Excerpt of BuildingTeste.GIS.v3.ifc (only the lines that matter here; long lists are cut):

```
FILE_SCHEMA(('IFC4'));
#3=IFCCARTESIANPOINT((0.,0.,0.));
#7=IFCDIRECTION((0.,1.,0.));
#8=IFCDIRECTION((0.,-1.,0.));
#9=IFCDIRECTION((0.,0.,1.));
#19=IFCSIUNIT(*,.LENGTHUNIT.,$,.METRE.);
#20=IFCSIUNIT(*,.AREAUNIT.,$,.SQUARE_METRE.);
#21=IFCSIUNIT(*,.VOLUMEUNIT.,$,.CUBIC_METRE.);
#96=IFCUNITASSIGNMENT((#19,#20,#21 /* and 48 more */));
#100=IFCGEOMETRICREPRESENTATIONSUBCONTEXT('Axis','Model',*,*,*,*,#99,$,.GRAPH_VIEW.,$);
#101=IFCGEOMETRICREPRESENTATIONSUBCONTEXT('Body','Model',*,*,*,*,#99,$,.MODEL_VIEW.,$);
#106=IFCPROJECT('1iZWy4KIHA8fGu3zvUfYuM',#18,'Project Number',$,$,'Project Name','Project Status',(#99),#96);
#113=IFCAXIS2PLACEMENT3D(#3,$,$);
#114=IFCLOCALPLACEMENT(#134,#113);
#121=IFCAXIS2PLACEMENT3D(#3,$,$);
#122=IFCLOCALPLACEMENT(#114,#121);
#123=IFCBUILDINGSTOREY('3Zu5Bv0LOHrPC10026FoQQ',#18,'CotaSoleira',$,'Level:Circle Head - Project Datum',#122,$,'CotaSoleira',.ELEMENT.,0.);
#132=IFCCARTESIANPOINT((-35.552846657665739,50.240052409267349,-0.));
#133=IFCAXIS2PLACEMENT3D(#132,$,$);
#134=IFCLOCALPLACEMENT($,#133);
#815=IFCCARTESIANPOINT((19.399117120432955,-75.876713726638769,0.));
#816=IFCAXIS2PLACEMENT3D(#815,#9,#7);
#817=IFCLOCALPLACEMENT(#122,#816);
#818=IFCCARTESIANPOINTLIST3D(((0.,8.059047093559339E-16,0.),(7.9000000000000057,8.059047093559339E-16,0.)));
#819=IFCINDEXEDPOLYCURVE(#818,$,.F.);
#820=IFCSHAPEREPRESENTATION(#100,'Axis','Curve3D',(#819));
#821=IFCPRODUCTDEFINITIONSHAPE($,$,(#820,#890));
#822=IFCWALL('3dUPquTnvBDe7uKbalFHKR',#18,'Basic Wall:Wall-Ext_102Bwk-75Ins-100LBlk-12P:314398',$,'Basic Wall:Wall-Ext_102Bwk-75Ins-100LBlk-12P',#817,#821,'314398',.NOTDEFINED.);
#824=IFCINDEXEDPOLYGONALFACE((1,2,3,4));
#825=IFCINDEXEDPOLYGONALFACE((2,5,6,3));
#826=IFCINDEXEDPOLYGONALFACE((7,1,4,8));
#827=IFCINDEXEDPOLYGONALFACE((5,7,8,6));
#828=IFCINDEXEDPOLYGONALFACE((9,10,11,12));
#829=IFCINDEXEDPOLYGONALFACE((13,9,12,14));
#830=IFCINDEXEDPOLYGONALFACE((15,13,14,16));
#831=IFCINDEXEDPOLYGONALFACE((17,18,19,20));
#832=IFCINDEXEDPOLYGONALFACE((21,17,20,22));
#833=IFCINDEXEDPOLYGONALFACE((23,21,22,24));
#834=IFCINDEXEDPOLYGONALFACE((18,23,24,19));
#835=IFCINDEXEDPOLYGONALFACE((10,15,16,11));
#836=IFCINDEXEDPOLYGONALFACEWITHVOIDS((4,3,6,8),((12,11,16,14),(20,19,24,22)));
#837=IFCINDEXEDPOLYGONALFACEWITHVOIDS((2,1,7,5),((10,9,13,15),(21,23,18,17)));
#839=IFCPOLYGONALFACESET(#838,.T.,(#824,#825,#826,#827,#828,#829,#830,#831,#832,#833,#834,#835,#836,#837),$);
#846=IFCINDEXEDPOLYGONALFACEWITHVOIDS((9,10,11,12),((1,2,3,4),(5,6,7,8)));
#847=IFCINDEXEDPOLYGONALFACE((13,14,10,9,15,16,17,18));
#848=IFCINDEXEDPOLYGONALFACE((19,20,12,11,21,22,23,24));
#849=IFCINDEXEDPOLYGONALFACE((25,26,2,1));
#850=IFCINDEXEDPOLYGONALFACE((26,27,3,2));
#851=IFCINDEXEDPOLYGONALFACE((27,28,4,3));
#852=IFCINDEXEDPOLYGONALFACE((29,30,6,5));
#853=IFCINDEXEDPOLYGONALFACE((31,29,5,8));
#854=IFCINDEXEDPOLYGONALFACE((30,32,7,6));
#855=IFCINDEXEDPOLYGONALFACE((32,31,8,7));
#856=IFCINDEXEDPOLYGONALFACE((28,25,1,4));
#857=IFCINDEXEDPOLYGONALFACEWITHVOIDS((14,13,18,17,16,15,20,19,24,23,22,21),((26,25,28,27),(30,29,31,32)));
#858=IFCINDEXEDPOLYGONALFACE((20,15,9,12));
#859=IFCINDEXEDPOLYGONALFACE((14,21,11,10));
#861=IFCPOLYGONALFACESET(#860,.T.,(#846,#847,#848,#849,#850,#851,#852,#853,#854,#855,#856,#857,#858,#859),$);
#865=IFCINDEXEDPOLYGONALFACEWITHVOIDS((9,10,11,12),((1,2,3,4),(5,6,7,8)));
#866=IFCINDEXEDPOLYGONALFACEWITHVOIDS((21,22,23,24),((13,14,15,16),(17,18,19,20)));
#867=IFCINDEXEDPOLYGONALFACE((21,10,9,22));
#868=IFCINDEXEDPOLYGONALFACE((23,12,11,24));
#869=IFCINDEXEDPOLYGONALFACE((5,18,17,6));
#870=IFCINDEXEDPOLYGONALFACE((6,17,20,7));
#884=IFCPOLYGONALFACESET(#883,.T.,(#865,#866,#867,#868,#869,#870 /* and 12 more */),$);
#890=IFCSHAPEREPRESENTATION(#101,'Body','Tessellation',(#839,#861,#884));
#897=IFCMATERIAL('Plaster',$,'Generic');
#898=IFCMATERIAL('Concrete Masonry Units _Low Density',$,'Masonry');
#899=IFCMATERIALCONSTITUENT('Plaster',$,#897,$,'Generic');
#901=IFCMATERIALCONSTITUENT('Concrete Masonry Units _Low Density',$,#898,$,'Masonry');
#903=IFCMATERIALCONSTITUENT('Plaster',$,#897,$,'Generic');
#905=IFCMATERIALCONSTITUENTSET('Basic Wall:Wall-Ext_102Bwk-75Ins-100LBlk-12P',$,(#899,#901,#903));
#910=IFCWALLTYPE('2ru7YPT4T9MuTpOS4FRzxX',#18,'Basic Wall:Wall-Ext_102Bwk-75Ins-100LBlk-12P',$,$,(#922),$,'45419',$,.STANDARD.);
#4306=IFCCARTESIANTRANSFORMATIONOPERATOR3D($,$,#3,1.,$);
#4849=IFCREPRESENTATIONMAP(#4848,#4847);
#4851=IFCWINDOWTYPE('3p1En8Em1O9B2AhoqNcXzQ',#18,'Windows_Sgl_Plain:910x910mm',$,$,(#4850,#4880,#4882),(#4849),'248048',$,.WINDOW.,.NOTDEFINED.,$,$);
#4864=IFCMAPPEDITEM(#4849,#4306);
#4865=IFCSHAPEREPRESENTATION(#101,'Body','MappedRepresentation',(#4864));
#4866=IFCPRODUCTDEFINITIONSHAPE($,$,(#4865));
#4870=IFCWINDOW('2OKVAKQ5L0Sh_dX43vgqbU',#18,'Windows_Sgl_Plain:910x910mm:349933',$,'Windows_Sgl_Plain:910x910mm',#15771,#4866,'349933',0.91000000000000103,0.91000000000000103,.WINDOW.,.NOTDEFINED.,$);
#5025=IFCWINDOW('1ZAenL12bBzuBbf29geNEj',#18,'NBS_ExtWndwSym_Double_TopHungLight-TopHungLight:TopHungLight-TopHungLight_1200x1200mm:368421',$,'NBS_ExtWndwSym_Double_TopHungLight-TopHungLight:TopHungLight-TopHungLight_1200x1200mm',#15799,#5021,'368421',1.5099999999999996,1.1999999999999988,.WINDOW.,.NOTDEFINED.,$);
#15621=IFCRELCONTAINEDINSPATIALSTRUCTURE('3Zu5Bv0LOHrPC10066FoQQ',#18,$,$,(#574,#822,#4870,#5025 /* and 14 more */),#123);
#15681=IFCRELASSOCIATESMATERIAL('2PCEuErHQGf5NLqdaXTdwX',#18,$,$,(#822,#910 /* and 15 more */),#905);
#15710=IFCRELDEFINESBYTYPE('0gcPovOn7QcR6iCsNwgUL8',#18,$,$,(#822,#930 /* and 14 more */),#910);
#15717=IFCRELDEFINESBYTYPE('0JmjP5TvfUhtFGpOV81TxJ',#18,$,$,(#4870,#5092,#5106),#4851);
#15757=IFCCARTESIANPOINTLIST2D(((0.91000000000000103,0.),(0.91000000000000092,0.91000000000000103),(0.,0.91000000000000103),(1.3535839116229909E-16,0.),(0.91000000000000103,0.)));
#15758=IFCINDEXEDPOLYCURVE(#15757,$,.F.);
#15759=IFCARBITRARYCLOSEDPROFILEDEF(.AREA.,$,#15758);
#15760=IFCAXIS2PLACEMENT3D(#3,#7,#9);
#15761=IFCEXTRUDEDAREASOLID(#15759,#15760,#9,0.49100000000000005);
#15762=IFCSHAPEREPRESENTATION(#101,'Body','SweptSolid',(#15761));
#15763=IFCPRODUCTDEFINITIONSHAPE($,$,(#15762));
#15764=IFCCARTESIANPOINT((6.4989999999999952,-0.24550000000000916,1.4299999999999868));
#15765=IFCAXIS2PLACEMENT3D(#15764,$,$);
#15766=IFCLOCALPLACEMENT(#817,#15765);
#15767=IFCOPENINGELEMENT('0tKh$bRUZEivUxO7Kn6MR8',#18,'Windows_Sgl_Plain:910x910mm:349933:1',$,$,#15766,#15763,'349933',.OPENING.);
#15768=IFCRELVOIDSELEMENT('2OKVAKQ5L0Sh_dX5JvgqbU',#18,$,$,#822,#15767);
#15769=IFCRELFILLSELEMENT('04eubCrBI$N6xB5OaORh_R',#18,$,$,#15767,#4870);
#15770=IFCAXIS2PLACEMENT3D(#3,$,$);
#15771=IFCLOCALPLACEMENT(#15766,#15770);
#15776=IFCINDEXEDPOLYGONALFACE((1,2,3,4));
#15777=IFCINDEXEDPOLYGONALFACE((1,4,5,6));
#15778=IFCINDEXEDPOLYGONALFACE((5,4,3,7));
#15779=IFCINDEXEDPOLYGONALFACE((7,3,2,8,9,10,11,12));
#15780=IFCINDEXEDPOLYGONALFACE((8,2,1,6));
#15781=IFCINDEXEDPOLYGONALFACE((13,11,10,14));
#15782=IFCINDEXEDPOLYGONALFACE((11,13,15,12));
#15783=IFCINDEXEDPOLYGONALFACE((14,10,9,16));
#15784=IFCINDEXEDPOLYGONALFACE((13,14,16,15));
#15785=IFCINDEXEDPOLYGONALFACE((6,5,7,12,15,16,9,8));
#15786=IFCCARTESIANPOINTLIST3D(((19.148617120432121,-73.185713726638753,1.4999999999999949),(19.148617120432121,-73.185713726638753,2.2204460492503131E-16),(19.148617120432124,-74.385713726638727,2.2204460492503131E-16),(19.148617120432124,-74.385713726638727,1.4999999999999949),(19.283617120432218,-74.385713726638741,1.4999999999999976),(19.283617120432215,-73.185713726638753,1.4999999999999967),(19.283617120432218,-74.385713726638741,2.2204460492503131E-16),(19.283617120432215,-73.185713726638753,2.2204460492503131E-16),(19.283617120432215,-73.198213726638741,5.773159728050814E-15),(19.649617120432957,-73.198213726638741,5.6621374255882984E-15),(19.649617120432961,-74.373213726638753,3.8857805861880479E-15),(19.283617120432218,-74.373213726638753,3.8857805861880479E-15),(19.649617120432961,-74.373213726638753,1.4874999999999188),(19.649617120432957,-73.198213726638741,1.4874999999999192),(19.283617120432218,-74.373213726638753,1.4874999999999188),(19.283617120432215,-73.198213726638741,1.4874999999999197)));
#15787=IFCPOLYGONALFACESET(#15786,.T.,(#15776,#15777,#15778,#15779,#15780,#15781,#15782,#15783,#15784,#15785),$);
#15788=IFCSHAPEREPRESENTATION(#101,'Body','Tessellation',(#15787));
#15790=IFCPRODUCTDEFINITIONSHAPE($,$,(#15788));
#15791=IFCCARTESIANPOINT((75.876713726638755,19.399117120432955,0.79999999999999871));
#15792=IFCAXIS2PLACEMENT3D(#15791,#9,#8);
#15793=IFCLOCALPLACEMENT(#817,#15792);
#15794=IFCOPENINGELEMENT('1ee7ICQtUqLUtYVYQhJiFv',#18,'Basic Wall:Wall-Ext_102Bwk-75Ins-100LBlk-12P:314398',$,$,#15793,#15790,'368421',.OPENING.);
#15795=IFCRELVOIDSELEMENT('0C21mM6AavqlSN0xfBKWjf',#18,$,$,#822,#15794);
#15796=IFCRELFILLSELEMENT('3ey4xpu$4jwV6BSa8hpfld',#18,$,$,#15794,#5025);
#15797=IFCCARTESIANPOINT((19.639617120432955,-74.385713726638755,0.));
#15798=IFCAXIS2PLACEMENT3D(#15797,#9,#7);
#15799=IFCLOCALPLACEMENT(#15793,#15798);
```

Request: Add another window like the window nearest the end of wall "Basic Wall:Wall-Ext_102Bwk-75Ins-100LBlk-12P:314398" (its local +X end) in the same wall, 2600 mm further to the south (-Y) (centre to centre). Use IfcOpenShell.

```python
import ifcopenshell
import ifcopenshell.api.feature
import ifcopenshell.api.geometry
import ifcopenshell.api.root
import ifcopenshell.geom
import ifcopenshell.util.element
import ifcopenshell.util.placement
import ifcopenshell.util.shape

model = ifcopenshell.open("BuildingTeste.GIS.v3.ifc")
settings = ifcopenshell.geom.settings()


def volume(element):
    """Net volume in cubic metres, openings subtracted."""
    shape = ifcopenshell.geom.create_shape(settings, element)
    return ifcopenshell.util.shape.get_volume(shape.geometry)


def reuse_history(source, copy):
    """copy_class also copies each property set's owner history, people and application; keep the originals."""
    for rel in copy.IsDefinedBy:
        if rel.is_a("IfcRelDefinesByProperties") and (history := rel.RelatingPropertyDefinition.OwnerHistory):
            rel.RelatingPropertyDefinition.OwnerHistory = source.OwnerHistory
            ifcopenshell.util.element.remove_deep2(model, history)


window = model.by_id(4870)
opening = window.FillsVoids[0].RelatingOpeningElement
wall = opening.VoidsElements[0].RelatingBuildingElement
before = volume(wall)
shift = ifcopenshell.util.placement.get_local_placement(wall.ObjectPlacement)[:3, 0] * -2.6

# copy_class copies the void relationship, type, container and properties, but no geometry.
new_opening = ifcopenshell.api.root.copy_class(model, product=opening)
new_opening.Representation = ifcopenshell.util.element.copy_deep(
    model, opening.Representation, exclude=["IfcGeometricRepresentationContext", "IfcRepresentationMap"]
)
new_opening.Name = "Windows_Sgl_Plain:910x910mm"
new_opening.Tag = None
new_window = ifcopenshell.api.root.copy_class(model, product=window)
new_window.Representation = ifcopenshell.util.element.copy_deep(
    model, window.Representation, exclude=["IfcGeometricRepresentationContext", "IfcRepresentationMap"]
)
new_window.Name = "Windows_Sgl_Plain:910x910mm"
new_window.Tag = None
reuse_history(window, new_window)
ifcopenshell.api.feature.add_filling(model, opening=new_opening, element=new_window)

for old, new in ((opening, new_opening), (window, new_window)):
    matrix = ifcopenshell.util.placement.get_local_placement(old.ObjectPlacement)
    matrix[:3, 3] += shift
    ifcopenshell.api.geometry.edit_object_placement(model, product=new, matrix=matrix, is_si=False)

after = volume(wall)

print(f"wall volume {before:.3f} -> {after:.3f} m3")

model.write("BuildingTeste.GIS.v3_rev.ifc")
```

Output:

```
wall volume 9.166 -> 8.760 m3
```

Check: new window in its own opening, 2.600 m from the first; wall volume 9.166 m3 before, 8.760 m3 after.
